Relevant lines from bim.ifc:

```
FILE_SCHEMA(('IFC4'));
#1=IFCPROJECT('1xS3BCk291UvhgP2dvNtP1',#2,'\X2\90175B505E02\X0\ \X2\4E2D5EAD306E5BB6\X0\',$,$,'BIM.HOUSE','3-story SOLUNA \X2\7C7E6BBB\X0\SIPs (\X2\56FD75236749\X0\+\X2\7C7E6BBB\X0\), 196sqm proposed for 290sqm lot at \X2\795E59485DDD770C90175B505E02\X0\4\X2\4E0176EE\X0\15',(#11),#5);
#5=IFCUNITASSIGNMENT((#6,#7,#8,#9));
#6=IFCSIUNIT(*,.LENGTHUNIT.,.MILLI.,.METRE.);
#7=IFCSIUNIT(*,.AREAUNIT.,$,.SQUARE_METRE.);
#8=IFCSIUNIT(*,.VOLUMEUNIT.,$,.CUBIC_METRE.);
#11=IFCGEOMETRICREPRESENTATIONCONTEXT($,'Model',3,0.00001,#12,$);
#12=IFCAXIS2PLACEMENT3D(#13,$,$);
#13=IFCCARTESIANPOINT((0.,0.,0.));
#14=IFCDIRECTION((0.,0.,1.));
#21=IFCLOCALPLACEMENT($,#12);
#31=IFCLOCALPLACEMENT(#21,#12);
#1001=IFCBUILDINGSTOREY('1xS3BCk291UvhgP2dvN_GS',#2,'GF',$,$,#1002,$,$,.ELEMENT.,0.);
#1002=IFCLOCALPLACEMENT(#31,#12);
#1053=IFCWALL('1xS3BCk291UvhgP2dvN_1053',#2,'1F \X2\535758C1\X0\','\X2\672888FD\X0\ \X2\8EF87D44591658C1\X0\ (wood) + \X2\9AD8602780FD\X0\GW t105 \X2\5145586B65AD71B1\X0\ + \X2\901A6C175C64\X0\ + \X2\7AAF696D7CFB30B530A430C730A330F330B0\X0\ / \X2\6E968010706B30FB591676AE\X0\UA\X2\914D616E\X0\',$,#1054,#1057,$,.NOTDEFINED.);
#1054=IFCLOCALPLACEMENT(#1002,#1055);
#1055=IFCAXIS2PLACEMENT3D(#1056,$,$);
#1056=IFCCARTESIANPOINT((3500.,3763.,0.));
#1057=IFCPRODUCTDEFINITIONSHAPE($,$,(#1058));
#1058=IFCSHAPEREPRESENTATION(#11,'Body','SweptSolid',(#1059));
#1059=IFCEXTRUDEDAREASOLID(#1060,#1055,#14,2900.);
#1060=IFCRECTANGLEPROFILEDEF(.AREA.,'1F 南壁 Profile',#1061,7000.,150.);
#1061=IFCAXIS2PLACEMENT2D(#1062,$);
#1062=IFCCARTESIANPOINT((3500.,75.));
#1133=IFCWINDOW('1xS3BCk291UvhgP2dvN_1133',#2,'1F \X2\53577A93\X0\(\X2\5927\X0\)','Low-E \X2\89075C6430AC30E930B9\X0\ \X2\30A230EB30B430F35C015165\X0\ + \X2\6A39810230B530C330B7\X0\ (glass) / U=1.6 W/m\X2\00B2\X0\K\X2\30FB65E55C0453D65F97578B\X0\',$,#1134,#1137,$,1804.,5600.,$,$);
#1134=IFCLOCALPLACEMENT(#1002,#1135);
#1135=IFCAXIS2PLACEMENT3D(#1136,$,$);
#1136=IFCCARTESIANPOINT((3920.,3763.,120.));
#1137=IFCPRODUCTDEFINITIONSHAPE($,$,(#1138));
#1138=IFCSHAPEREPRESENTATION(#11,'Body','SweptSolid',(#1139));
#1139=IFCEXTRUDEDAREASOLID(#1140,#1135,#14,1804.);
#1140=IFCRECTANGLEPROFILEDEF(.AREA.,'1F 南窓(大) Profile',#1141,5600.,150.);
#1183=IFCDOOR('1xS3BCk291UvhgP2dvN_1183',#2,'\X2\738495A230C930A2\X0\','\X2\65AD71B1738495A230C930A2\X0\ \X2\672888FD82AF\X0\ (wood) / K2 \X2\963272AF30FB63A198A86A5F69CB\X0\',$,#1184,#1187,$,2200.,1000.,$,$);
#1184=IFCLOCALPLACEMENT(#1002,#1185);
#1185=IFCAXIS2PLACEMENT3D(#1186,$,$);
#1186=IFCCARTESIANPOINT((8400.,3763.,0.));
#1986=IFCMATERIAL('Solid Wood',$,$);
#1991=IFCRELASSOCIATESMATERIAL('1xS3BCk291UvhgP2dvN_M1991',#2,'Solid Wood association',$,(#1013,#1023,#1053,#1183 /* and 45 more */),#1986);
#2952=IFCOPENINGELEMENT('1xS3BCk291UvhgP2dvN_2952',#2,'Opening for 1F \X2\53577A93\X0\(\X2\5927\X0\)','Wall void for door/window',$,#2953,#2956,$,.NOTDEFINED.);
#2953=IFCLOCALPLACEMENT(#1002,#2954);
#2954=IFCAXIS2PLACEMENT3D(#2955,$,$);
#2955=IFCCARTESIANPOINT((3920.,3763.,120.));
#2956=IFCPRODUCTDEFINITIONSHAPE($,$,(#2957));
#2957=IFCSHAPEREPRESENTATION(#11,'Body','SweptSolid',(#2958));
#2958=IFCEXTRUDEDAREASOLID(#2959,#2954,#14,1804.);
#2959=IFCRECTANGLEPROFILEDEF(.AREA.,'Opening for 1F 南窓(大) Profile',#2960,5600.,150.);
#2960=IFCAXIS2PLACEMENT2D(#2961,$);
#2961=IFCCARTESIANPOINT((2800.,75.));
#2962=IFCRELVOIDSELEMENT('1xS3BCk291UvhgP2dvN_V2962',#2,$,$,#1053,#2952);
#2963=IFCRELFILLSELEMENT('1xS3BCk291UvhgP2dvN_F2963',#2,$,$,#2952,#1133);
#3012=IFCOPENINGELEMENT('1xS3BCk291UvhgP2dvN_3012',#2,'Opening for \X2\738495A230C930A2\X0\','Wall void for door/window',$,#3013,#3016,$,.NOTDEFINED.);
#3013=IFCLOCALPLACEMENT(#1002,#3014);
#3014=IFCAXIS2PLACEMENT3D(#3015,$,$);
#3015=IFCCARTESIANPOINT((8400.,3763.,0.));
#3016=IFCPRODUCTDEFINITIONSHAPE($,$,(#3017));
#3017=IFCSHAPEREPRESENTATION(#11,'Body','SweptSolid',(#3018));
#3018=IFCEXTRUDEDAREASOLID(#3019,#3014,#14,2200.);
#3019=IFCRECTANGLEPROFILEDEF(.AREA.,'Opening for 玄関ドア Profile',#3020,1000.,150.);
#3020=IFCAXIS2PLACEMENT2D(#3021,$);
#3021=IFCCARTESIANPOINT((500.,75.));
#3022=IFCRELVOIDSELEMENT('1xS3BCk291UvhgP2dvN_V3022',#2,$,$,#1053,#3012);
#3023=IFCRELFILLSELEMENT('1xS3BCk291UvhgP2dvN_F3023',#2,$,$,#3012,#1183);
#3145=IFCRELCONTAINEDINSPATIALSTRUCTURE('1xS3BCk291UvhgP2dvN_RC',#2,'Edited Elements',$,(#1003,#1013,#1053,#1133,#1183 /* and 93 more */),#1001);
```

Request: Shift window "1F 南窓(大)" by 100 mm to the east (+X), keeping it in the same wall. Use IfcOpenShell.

```python
import ifcopenshell
import ifcopenshell.api.geometry
import ifcopenshell.util.placement

model = ifcopenshell.open("bim.ifc")

window = model.by_id(1133)
opening = window.FillsVoids[0].RelatingOpeningElement
wall = opening.VoidsElements[0].RelatingBuildingElement

wall_matrix = ifcopenshell.util.placement.get_local_placement(wall.ObjectPlacement)
shift = wall_matrix[:3, 0] * 100.0
before = ifcopenshell.util.placement.get_local_placement(window.ObjectPlacement)[:3, 3].copy()

# The window is not placed relative to its opening, so move both.
for product in (opening, window):
    matrix = ifcopenshell.util.placement.get_local_placement(product.ObjectPlacement)
    matrix[:3, 3] += shift
    ifcopenshell.api.geometry.edit_object_placement(model, product=product, matrix=matrix, is_si=False)

after = ifcopenshell.util.placement.get_local_placement(window.ObjectPlacement)[:3, 3]
print("window moved by", (after - before).round(3) + 0.0)

model.write("bim_v2.ifc")
```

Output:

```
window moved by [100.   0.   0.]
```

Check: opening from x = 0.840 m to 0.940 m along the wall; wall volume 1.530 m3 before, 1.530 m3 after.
